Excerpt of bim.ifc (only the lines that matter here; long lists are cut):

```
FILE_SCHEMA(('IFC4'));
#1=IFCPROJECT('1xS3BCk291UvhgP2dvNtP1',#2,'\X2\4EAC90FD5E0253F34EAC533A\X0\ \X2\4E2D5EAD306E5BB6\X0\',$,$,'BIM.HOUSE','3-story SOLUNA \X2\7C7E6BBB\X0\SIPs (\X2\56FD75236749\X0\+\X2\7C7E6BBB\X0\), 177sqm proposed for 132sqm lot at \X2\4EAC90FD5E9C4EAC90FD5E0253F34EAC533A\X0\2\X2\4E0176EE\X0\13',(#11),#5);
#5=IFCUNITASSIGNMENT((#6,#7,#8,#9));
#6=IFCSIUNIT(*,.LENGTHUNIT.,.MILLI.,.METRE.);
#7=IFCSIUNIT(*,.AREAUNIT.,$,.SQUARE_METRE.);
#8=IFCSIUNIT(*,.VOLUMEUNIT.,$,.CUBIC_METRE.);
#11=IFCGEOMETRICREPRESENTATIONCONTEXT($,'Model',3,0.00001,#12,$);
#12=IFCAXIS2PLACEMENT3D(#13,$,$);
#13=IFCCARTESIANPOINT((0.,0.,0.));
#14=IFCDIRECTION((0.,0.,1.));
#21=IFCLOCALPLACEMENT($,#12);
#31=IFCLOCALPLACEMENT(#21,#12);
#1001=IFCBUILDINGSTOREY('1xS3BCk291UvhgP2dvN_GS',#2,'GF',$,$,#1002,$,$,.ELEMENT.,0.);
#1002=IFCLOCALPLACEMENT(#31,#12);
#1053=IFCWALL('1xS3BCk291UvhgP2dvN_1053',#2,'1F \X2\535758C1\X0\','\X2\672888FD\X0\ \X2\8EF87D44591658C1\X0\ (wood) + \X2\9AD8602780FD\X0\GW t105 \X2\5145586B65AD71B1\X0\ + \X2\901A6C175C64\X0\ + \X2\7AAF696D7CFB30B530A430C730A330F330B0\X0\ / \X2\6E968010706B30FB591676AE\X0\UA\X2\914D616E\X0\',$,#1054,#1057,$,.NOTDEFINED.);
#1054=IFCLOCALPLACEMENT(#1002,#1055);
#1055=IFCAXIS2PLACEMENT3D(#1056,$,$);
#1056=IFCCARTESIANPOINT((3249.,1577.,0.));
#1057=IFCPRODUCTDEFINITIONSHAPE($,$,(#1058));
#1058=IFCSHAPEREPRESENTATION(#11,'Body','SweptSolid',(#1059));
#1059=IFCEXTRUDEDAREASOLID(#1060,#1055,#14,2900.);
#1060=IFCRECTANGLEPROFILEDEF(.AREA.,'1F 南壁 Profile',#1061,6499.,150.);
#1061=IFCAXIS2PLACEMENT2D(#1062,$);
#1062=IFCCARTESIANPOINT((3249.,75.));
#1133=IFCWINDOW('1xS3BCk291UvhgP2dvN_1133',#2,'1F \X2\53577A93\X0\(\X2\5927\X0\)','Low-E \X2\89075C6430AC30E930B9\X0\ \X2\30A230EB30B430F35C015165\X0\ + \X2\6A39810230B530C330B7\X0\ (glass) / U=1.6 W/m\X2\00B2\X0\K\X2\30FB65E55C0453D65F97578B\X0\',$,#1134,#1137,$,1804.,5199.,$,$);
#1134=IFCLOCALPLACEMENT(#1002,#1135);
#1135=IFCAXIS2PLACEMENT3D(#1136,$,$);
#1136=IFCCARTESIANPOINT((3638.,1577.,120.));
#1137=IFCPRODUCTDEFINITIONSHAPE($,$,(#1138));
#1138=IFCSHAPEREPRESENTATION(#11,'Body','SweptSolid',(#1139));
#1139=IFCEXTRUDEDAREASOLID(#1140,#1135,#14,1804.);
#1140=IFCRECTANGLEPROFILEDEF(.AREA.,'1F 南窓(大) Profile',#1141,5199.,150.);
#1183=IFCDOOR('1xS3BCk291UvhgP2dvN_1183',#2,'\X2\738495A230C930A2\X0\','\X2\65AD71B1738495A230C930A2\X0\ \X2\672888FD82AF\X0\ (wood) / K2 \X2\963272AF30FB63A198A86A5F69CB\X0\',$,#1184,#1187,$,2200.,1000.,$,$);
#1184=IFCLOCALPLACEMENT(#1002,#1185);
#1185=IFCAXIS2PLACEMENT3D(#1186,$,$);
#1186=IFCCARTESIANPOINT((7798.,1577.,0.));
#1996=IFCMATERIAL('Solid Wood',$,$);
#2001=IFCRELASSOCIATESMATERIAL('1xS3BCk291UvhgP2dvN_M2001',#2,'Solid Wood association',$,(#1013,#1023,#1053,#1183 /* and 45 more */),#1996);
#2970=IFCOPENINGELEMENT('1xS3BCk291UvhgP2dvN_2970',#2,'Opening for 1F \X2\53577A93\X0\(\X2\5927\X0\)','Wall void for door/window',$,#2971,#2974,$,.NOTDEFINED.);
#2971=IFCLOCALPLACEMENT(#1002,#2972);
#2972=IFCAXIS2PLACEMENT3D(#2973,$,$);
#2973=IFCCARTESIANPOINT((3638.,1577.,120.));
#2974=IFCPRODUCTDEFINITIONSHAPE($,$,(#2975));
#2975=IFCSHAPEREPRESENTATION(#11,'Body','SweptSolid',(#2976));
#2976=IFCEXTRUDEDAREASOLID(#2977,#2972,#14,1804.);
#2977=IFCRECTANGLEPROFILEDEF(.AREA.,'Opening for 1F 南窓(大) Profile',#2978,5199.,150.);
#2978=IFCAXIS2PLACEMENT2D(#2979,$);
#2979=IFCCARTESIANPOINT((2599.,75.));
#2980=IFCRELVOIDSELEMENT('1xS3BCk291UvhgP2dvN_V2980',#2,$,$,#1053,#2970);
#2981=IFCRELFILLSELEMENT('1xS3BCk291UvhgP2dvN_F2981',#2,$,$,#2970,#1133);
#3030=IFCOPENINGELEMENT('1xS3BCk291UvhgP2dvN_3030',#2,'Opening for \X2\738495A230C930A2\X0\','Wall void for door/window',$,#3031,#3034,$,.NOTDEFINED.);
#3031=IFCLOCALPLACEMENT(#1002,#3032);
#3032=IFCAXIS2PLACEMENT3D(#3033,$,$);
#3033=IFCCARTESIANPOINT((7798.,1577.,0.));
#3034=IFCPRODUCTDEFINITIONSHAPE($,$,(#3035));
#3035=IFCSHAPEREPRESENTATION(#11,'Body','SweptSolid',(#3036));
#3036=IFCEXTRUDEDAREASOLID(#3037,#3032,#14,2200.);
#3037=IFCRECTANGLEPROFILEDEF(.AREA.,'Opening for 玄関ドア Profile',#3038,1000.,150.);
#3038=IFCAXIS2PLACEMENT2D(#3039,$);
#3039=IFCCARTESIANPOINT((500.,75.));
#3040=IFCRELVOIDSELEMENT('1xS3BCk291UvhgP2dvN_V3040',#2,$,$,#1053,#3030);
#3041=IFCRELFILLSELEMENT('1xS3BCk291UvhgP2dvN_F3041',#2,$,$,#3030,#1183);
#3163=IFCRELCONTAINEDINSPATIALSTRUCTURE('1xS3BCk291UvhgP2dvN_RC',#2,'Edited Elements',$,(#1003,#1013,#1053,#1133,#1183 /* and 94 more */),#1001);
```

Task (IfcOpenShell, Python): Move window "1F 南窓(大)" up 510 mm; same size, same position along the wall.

```python
import numpy as np
import ifcopenshell
import ifcopenshell.api.geometry
import ifcopenshell.util.placement
import ifcopenshell.util.unit

model = ifcopenshell.open("bim.ifc")
unit_scale = ifcopenshell.util.unit.calculate_unit_scale(model)

window = model.by_guid("1xS3BCk291UvhgP2dvN_1133")
opening = window.FillsVoids[0].RelatingOpeningElement
dz = 0.51 / unit_scale

shift = np.array([0.0, 0.0, dz])
# The window is not placed relative to its opening, so move both.
for product in (opening, window):
    matrix = ifcopenshell.util.placement.get_local_placement(product.ObjectPlacement)
    matrix[:3, 3] += shift
    ifcopenshell.api.geometry.edit_object_placement(model, product=product, matrix=matrix, is_si=False)

print(f"moved by {dz * unit_scale:+.3f} m")

model.write("bim_edited.ifc")
```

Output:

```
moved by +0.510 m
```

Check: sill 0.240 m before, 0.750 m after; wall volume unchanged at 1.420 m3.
